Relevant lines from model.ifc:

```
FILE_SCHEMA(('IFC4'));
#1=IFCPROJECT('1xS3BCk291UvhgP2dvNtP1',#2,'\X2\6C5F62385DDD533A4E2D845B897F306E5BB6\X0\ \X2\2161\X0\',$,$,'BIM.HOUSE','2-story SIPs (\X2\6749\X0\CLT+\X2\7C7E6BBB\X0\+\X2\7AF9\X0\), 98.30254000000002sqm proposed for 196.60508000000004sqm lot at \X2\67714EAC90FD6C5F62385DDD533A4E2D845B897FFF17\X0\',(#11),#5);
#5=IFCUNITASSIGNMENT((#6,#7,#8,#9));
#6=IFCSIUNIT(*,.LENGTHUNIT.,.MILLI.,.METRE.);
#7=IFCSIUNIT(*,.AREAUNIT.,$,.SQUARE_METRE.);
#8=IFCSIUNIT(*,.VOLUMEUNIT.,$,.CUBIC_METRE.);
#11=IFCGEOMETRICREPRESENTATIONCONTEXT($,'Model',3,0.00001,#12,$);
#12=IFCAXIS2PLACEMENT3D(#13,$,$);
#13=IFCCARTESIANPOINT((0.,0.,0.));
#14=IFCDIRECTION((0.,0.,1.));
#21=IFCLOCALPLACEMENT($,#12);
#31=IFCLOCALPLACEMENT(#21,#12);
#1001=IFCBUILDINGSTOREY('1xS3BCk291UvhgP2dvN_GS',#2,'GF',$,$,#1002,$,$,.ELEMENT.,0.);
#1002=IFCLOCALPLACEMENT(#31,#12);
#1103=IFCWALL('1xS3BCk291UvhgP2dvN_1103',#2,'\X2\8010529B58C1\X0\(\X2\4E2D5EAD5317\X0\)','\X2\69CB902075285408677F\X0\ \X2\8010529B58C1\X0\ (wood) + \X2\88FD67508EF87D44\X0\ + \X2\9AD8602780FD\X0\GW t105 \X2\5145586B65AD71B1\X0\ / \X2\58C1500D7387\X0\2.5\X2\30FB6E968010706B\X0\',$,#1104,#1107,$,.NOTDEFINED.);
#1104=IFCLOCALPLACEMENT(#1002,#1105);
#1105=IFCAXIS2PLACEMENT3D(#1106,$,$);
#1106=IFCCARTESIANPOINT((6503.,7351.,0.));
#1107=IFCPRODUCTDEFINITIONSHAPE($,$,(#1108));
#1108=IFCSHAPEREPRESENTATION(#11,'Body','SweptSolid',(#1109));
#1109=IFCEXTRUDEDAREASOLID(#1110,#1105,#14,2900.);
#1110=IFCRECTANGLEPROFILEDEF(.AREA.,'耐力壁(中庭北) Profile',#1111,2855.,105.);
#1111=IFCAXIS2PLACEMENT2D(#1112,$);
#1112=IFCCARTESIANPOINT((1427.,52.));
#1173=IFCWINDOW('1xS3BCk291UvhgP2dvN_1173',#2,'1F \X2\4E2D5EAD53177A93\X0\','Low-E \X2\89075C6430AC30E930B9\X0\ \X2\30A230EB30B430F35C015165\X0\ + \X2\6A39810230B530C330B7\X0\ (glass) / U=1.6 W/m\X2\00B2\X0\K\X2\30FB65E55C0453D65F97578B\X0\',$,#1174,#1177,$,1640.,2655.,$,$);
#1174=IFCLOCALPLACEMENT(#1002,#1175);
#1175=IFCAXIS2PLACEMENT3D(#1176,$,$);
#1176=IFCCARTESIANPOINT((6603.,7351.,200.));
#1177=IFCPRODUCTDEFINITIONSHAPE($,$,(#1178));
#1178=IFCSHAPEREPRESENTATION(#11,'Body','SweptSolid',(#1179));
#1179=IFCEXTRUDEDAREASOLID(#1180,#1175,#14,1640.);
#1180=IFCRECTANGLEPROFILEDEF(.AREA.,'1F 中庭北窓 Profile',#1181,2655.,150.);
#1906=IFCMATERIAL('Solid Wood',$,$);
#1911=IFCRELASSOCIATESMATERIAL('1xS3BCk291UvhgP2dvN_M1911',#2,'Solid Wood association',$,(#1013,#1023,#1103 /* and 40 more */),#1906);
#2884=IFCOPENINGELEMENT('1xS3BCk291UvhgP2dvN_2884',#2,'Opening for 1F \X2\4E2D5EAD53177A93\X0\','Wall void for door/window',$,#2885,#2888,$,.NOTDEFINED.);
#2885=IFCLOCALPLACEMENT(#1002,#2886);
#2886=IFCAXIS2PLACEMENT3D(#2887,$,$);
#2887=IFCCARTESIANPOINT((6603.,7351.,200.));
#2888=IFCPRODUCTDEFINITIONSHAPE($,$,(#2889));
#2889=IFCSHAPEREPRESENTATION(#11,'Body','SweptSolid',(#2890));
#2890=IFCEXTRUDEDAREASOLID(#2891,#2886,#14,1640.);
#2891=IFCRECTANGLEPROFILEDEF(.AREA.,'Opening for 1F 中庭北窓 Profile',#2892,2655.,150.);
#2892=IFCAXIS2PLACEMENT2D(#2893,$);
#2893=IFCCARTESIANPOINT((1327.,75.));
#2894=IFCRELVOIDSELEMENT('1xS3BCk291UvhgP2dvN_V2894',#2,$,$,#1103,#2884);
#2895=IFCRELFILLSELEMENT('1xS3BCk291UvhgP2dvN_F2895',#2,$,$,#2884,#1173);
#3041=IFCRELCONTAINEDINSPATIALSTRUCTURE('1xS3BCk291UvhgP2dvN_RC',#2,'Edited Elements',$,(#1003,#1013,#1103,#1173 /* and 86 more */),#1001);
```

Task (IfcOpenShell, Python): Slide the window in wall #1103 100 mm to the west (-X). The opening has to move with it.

```python
import ifcopenshell
import ifcopenshell.api.geometry
import ifcopenshell.util.placement
import ifcopenshell.util.unit

model = ifcopenshell.open("model.ifc")
unit_scale = ifcopenshell.util.unit.calculate_unit_scale(model)

window = model.by_id(1173)
opening = window.FillsVoids[0].RelatingOpeningElement
wall = opening.VoidsElements[0].RelatingBuildingElement

wall_matrix = ifcopenshell.util.placement.get_local_placement(wall.ObjectPlacement)
shift = wall_matrix[:3, 0] * -0.1 / unit_scale
before = ifcopenshell.util.placement.get_local_placement(window.ObjectPlacement)[:3, 3].copy()

# The window is not placed relative to its opening, so move both.
for product in (opening, window):
    matrix = ifcopenshell.util.placement.get_local_placement(product.ObjectPlacement)
    matrix[:3, 3] += shift
    ifcopenshell.api.geometry.edit_object_placement(model, product=product, matrix=matrix, is_si=False)

after = ifcopenshell.util.placement.get_local_placement(window.ObjectPlacement)[:3, 3]
print("window moved by", (after - before).round(3) + 0.0)

model.write("model-out.ifc")
```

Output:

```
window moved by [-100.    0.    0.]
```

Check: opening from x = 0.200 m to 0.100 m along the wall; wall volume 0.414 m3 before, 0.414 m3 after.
